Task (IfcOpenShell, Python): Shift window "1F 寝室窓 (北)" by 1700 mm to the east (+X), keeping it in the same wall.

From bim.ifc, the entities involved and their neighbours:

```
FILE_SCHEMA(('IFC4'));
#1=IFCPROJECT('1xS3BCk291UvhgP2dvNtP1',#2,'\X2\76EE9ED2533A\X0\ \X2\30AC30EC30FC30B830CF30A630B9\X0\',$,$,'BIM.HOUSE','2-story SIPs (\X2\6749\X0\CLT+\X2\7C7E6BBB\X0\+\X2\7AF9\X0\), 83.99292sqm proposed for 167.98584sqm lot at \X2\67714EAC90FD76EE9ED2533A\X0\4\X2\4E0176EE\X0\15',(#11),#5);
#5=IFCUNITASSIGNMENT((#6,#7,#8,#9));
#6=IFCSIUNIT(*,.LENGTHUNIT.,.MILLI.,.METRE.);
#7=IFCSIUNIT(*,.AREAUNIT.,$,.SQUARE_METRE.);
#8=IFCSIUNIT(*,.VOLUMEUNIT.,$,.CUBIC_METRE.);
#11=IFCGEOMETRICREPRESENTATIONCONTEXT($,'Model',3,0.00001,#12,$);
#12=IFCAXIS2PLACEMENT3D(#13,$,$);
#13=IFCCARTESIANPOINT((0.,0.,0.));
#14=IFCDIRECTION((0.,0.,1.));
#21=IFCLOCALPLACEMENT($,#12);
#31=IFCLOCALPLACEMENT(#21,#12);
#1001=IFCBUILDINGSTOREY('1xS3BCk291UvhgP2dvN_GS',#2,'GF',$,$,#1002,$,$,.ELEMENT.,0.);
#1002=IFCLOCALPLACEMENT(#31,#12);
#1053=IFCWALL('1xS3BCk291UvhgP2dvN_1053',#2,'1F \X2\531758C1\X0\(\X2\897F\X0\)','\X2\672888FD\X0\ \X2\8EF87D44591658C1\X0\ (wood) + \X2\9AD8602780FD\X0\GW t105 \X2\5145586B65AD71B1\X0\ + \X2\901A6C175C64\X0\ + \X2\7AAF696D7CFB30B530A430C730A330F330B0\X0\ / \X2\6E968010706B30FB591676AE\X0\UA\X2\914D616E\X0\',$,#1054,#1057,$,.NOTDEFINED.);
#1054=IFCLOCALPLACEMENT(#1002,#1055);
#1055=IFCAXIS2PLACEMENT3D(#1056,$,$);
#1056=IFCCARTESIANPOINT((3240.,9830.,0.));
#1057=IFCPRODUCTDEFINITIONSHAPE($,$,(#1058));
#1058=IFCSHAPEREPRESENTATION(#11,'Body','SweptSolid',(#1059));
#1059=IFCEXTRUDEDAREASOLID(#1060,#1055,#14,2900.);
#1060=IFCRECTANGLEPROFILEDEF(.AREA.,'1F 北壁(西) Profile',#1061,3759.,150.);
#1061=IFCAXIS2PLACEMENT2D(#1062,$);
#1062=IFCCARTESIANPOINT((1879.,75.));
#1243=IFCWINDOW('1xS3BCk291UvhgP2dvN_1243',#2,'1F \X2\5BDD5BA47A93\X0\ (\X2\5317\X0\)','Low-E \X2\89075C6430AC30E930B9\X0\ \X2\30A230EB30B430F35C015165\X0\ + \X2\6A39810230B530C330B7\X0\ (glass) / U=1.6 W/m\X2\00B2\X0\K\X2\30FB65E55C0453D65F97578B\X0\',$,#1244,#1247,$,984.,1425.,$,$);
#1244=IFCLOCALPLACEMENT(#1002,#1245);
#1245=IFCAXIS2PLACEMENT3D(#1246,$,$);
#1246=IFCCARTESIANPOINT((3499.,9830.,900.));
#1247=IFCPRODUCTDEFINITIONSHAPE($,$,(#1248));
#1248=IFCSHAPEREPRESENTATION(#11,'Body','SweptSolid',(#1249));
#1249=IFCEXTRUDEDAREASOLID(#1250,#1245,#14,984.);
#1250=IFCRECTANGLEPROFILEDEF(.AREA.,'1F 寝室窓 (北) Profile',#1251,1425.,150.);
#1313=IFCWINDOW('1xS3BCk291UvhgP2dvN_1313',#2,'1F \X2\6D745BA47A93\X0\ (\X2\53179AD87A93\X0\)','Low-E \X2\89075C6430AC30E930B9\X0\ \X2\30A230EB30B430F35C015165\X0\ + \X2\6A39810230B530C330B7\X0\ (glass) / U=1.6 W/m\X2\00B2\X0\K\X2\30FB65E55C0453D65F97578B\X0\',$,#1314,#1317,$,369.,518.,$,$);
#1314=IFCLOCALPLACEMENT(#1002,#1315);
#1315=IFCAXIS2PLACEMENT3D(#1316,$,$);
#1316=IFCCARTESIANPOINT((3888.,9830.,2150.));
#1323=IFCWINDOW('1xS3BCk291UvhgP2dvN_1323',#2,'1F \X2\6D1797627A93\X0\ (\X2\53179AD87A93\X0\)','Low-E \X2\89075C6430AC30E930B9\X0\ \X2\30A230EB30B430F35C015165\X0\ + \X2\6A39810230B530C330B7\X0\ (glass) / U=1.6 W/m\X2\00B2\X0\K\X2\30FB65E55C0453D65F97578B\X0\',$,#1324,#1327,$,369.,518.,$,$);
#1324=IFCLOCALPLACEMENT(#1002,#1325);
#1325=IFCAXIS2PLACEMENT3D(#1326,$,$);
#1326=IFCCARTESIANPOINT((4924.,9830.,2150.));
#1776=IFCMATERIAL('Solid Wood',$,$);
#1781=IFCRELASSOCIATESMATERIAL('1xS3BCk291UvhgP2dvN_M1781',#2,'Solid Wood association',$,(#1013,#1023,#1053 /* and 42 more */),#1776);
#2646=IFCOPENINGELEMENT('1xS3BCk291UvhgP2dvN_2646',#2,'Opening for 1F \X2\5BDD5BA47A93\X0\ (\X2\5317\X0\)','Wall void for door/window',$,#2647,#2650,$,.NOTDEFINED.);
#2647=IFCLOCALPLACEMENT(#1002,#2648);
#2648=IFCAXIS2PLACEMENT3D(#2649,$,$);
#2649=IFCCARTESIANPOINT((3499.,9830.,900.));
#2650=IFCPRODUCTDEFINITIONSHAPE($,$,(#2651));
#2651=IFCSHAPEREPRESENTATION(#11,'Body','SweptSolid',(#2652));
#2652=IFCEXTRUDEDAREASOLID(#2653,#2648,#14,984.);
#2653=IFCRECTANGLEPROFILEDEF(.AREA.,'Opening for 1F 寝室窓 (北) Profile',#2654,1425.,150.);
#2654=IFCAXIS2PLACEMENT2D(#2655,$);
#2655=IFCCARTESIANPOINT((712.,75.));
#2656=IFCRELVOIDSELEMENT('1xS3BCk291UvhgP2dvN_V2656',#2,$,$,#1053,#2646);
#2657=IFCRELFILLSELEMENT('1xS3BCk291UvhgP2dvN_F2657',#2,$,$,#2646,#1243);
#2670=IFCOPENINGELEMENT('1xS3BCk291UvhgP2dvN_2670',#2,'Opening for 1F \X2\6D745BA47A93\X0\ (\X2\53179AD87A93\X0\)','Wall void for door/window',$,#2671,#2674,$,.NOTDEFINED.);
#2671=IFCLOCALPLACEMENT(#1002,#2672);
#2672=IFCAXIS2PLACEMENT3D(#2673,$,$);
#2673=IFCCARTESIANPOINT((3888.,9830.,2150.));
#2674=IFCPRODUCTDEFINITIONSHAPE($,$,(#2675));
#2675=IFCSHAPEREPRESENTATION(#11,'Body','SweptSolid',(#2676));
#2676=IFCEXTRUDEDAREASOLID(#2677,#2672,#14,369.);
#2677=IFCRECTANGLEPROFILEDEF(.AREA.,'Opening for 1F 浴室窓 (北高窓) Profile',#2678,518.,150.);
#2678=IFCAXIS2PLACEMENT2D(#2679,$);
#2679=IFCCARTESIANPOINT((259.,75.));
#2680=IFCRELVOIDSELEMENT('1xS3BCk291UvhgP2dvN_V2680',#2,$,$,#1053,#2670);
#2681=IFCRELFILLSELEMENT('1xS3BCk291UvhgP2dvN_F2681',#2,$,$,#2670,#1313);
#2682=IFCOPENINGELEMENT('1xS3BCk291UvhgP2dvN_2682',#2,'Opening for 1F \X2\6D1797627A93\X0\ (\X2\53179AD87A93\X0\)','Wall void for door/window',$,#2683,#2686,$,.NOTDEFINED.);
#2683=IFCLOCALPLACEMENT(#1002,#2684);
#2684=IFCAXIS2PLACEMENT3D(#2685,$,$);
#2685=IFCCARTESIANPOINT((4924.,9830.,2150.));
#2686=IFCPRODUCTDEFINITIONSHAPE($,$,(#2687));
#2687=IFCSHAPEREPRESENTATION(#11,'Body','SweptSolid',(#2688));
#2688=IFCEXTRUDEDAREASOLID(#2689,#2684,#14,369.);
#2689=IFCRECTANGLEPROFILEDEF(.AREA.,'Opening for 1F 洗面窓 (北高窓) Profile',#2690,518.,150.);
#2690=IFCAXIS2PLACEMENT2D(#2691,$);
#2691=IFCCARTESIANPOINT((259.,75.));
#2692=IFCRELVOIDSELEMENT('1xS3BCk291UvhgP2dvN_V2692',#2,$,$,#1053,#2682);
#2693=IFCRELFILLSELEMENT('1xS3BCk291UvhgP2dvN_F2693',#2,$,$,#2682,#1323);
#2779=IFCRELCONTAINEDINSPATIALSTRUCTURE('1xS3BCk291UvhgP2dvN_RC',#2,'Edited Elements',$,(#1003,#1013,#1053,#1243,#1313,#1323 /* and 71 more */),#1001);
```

```python
import ifcopenshell
import ifcopenshell.api.geometry
import ifcopenshell.util.placement
import ifcopenshell.util.unit

model = ifcopenshell.open("bim.ifc")
unit_scale = ifcopenshell.util.unit.calculate_unit_scale(model)

window = model.by_guid("1xS3BCk291UvhgP2dvN_1243")
opening = window.FillsVoids[0].RelatingOpeningElement
wall = opening.VoidsElements[0].RelatingBuildingElement

wall_matrix = ifcopenshell.util.placement.get_local_placement(wall.ObjectPlacement)
shift = wall_matrix[:3, 0] * 1.7 / unit_scale
before = ifcopenshell.util.placement.get_local_placement(window.ObjectPlacement)[:3, 3].copy()

# The window is not placed relative to its opening, so move both.
for product in (opening, window):
    matrix = ifcopenshell.util.placement.get_local_placement(product.ObjectPlacement)
    matrix[:3, 3] += shift
    ifcopenshell.api.geometry.edit_object_placement(model, product=product, matrix=matrix, is_si=False)

after = ifcopenshell.util.placement.get_local_placement(window.ObjectPlacement)[:3, 3]
print("window moved by", (after - before).round(3) + 0.0)

model.write("bim-out.ifc")
```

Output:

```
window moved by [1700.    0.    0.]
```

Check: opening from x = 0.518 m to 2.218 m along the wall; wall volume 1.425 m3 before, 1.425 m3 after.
